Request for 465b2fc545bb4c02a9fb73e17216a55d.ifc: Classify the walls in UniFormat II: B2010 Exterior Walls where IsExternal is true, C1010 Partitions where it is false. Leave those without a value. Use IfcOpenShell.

First a look at what the model holds.

```python
import ifcopenshell
import ifcopenshell.util.element

model = ifcopenshell.open("465b2fc545bb4c02a9fb73e17216a55d.ifc")
print(model.schema)
print("classifications:", [c.Name for c in model.by_type("IfcClassification")])
values = [ifcopenshell.util.element.get_pset(e, "Pset_WallCommon", "IsExternal") for e in model.by_type("IfcWall")]
for value in (True, False, None):
    print("IsExternal", value, values.count(value))
```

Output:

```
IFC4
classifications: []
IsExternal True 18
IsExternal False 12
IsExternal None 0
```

```python
import ifcopenshell
import ifcopenshell.api.classification
import ifcopenshell.util.element

model = ifcopenshell.open("465b2fc545bb4c02a9fb73e17216a55d.ifc")

system = ifcopenshell.api.classification.add_classification(model, classification="UniFormat II")

walls = model.by_type("IfcWall")
external = {e: ifcopenshell.util.element.get_pset(e, "Pset_WallCommon", "IsExternal") for e in walls}
for flag, code, name in ((True, "B2010", "Exterior Walls"), (False, "C1010", "Partitions")):
    products = [e for e in walls if external[e] is flag]
    ifcopenshell.api.classification.add_reference(
        model, products=products, classification=system, identification=code, name=name
    )
    print(code, len(products))

model.write("465b2fc545bb4c02a9fb73e17216a55d_updated.ifc")
```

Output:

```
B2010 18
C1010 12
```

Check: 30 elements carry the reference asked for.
